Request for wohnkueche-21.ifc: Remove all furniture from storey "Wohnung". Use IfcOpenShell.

First a look at what the model holds.

```python
import ifcopenshell
import ifcopenshell.util.element

model = ifcopenshell.open("wohnkueche-21.ifc")
print(model.schema)
storey = next(s for s in model.by_type("IfcBuildingStorey") if s.Name == "Wohnung")
furniture = [e for e in ifcopenshell.util.element.get_decomposition(storey) if e.is_a("IfcFurnishingElement")]
seen = {}
for e in furniture:
    element_type = ifcopenshell.util.element.get_type(e)
    name = element_type.Name if element_type not in (None, e) else None
    seen[name] = seen.get(name, 0) + 1
for name, count in sorted(seen.items(), key=str):
    print(count, "x", name)
```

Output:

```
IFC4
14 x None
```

```python
import ifcopenshell
import ifcopenshell.api.root
import ifcopenshell.util.element

model = ifcopenshell.open("wohnkueche-21.ifc")

storey = next(s for s in model.by_type("IfcBuildingStorey") if s.Name == "Wohnung")
furniture = [e for e in ifcopenshell.util.element.get_decomposition(storey) if e.is_a("IfcFurnishingElement")]

for e in furniture:
    ifcopenshell.api.root.remove_product(model, product=e)
print(len(furniture), "removed")

model.write("wohnkueche-21_edited.ifc")
```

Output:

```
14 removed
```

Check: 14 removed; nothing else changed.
